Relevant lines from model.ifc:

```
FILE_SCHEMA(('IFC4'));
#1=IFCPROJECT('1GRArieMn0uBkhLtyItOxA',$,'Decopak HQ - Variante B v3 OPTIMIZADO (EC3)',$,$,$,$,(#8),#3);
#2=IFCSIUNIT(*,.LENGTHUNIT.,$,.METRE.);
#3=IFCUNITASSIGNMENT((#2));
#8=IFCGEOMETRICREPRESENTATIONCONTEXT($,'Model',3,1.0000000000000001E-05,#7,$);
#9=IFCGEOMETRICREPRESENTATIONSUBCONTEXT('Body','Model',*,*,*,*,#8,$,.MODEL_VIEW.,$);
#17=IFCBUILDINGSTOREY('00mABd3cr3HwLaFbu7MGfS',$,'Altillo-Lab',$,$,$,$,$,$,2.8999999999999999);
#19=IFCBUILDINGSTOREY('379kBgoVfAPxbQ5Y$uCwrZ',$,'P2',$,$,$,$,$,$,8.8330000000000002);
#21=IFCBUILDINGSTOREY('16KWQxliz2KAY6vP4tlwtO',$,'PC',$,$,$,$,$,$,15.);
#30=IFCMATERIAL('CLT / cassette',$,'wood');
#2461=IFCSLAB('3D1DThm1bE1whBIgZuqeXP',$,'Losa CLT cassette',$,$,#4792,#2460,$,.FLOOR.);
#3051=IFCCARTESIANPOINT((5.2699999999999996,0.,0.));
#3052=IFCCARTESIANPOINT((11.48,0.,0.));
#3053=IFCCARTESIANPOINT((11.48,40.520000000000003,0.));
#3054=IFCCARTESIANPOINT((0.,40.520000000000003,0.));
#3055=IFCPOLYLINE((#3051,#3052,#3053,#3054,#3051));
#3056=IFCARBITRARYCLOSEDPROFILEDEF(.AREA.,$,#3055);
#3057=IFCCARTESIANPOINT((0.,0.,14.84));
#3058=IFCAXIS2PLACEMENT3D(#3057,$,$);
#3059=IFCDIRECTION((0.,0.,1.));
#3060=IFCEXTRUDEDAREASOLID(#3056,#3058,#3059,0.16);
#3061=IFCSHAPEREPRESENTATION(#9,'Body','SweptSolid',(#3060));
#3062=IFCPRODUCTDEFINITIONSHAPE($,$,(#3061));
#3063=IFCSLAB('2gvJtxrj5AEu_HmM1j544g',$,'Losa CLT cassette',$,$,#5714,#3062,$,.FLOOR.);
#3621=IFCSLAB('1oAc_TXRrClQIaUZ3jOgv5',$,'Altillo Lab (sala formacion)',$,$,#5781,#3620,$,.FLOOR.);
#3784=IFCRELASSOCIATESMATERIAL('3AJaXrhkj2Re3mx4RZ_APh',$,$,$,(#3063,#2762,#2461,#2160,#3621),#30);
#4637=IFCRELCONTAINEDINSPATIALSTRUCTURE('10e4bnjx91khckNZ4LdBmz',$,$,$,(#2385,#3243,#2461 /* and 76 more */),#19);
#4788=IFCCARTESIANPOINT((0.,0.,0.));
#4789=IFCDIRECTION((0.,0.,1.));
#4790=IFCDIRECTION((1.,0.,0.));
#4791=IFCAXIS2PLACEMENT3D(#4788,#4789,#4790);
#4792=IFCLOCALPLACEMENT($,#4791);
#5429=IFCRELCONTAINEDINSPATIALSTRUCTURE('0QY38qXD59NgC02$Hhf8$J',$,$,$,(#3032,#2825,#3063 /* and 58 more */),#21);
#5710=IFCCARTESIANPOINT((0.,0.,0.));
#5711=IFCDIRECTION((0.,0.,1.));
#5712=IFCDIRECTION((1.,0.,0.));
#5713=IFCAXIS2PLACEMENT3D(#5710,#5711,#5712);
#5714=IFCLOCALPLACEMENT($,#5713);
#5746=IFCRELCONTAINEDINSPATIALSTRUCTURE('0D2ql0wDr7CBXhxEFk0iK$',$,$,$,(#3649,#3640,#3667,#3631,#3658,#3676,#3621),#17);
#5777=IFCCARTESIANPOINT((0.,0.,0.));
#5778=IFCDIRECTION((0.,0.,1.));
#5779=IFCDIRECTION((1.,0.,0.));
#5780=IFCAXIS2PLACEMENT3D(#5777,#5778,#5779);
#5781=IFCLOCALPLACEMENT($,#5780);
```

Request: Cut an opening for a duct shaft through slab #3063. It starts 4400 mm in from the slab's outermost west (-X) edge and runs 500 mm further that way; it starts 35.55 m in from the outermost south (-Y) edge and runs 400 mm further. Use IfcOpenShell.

```python
import numpy as np
import ifcopenshell
import ifcopenshell.api.feature
import ifcopenshell.api.geometry
import ifcopenshell.api.root
import ifcopenshell.geom
import ifcopenshell.util.placement
import ifcopenshell.util.representation
import ifcopenshell.util.shape
import ifcopenshell.util.unit

model = ifcopenshell.open("model.ifc")
unit_scale = ifcopenshell.util.unit.calculate_unit_scale(model)
settings = ifcopenshell.geom.settings()


def volume(element):
    """Net volume in cubic metres, openings subtracted."""
    shape = ifcopenshell.geom.create_shape(settings, element)
    return ifcopenshell.util.shape.get_volume(shape.geometry)


slab = model.by_guid("2gvJtxrj5AEu_HmM1j544g")
before = volume(slab)

# Extent in the slab's own axes, in metres. The edges named are its -X and -Y sides.
slab_shape = ifcopenshell.geom.create_shape(settings, slab)
vertices = ifcopenshell.util.shape.get_vertices(slab_shape.geometry)
x_min, y_min, bottom = vertices.min(axis=0)
top = vertices[:, 2].max()

opening = ifcopenshell.api.root.create_entity(model, ifc_class="IfcOpeningElement", name="Duct shaft opening", predefined_type="OPENING")
context = ifcopenshell.util.representation.get_context(model, "Model", "Body", "MODEL_VIEW")
width, depth = 0.5, 0.4
outline = [(0.0, 0.0), (width, 0.0), (width, depth), (0.0, depth), (0.0, 0.0)]
# Overshoot both faces by 50 mm so the cut is clean.
shape = ifcopenshell.api.geometry.add_slab_representation(
    model, context=context, depth=top - bottom + 0.1, polyline=outline
)
ifcopenshell.api.geometry.assign_representation(model, product=opening, representation=shape)

matrix = ifcopenshell.util.placement.get_local_placement(slab.ObjectPlacement)
matrix[:, 3] = matrix @ np.append(np.array([x_min + 4.4, y_min + 35.55, bottom - 0.05]) / unit_scale, 1.0)
ifcopenshell.api.geometry.edit_object_placement(model, product=opening, matrix=matrix, is_si=False)
ifcopenshell.api.feature.add_feature(model, feature=opening, element=slab)

after = volume(slab)

print(f"slab volume {before:.3f} -> {after:.3f} m3")

model.write("model_rev.ifc")
```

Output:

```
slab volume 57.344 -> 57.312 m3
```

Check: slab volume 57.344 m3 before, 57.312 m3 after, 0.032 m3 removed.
